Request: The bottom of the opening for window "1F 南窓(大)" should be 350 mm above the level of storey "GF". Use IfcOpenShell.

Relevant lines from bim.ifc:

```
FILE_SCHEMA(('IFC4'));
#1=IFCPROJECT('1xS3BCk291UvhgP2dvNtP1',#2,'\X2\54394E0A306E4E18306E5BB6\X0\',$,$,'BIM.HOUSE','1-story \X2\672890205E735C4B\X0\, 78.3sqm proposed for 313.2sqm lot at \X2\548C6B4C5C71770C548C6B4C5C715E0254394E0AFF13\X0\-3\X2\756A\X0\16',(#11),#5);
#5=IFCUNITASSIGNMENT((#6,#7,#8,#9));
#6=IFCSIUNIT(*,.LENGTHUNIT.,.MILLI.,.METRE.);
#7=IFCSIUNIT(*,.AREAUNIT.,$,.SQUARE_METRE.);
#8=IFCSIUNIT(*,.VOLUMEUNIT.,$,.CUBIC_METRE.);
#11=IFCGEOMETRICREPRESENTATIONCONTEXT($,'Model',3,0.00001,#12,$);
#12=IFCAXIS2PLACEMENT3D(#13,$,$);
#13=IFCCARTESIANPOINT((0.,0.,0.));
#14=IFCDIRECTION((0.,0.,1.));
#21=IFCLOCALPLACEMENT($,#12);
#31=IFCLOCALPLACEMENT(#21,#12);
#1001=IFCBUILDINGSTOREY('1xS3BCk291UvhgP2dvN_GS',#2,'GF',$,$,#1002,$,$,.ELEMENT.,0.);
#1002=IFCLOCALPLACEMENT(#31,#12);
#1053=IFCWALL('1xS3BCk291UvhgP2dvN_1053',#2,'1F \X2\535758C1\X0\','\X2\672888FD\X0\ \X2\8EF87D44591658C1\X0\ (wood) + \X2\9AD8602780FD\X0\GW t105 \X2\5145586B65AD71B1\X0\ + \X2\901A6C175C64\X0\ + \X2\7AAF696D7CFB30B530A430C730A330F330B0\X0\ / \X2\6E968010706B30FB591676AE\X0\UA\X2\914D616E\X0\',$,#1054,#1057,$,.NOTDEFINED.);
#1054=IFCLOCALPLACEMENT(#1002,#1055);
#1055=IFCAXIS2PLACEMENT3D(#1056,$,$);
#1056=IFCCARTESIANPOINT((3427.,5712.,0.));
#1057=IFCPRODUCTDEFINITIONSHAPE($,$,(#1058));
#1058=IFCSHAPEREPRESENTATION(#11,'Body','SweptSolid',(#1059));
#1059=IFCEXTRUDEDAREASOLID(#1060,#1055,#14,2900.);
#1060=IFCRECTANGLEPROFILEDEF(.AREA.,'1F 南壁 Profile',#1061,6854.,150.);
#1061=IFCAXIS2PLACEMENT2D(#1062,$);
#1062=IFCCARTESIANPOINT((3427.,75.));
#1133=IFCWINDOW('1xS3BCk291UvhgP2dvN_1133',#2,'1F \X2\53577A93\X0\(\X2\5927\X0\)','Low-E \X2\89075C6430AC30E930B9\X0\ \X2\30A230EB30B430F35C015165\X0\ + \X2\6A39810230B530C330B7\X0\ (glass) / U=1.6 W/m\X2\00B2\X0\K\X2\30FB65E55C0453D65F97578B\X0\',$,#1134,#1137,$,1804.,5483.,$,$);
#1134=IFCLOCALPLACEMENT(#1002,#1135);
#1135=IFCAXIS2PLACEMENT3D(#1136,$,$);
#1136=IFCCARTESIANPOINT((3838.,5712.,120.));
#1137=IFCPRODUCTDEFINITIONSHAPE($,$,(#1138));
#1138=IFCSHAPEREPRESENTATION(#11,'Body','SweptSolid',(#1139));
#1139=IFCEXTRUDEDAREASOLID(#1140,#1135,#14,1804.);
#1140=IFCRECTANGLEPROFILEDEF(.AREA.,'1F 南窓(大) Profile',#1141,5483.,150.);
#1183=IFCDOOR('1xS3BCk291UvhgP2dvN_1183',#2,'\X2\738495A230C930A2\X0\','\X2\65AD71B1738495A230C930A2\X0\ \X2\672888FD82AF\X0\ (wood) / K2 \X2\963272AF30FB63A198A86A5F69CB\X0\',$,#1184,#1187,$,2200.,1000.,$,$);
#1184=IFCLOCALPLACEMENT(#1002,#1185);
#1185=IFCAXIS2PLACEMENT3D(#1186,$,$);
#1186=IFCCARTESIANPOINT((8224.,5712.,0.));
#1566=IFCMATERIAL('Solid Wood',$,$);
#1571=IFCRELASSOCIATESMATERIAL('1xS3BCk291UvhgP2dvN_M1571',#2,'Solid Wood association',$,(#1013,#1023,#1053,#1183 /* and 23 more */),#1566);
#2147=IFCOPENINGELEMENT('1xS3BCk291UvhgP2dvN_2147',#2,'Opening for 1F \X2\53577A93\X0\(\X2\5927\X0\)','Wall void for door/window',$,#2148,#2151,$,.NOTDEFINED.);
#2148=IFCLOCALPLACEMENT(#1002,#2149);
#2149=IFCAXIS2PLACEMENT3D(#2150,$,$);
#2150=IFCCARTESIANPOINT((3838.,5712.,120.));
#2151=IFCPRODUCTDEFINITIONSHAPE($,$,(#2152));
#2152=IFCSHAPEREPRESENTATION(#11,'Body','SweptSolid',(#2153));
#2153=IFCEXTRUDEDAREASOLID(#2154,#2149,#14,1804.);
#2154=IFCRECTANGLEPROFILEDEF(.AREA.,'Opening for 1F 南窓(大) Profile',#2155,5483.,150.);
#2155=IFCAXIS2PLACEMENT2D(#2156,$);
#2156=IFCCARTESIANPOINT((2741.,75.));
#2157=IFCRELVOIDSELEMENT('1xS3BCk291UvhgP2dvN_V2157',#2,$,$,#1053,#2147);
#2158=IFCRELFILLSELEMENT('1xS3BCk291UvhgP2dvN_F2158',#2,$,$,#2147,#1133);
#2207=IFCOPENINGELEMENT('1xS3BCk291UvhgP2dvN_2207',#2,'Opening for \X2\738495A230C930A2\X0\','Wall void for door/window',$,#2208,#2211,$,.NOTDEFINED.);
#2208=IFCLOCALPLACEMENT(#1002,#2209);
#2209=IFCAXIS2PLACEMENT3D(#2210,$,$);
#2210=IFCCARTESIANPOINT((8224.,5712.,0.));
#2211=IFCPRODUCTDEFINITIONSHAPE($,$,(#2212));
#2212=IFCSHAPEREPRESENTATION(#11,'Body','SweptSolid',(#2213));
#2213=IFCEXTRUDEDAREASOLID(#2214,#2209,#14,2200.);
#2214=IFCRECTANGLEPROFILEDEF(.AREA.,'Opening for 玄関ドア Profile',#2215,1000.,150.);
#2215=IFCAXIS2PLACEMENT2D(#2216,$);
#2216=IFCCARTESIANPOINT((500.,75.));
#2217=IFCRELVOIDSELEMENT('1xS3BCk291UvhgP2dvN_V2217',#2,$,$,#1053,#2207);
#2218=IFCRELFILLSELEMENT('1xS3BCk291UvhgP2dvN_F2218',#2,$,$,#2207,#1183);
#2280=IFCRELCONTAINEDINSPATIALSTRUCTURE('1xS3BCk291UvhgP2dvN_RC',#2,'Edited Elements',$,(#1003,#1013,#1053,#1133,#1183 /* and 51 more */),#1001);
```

```python
import numpy as np
import ifcopenshell
import ifcopenshell.api.geometry
import ifcopenshell.geom
import ifcopenshell.util.element
import ifcopenshell.util.placement
import ifcopenshell.util.shape
import ifcopenshell.util.unit

model = ifcopenshell.open("bim.ifc")
unit_scale = ifcopenshell.util.unit.calculate_unit_scale(model)

window = model.by_guid("1xS3BCk291UvhgP2dvN_1133")
opening = window.FillsVoids[0].RelatingOpeningElement
storey = ifcopenshell.util.element.get_container(window, ifc_class="IfcBuildingStorey")
level = ifcopenshell.util.placement.get_local_placement(storey.ObjectPlacement)[2, 3]

# The opening's origin need not be at the sill, so measure its lowest point.
shape = ifcopenshell.geom.create_shape(ifcopenshell.geom.settings(), opening)
bottom = ifcopenshell.util.shape.get_shape_bottom_elevation(shape, shape.geometry) / unit_scale
dz = level + 0.35 / unit_scale - bottom

shift = np.array([0.0, 0.0, dz])
# The window is not placed relative to its opening, so move both.
for product in (opening, window):
    matrix = ifcopenshell.util.placement.get_local_placement(product.ObjectPlacement)
    matrix[:3, 3] += shift
    ifcopenshell.api.geometry.edit_object_placement(model, product=product, matrix=matrix, is_si=False)

print(f"moved by {dz * unit_scale:+.3f} m")

model.write("bim_v2.ifc")
```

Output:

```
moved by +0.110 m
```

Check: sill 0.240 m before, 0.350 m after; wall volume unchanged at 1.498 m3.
